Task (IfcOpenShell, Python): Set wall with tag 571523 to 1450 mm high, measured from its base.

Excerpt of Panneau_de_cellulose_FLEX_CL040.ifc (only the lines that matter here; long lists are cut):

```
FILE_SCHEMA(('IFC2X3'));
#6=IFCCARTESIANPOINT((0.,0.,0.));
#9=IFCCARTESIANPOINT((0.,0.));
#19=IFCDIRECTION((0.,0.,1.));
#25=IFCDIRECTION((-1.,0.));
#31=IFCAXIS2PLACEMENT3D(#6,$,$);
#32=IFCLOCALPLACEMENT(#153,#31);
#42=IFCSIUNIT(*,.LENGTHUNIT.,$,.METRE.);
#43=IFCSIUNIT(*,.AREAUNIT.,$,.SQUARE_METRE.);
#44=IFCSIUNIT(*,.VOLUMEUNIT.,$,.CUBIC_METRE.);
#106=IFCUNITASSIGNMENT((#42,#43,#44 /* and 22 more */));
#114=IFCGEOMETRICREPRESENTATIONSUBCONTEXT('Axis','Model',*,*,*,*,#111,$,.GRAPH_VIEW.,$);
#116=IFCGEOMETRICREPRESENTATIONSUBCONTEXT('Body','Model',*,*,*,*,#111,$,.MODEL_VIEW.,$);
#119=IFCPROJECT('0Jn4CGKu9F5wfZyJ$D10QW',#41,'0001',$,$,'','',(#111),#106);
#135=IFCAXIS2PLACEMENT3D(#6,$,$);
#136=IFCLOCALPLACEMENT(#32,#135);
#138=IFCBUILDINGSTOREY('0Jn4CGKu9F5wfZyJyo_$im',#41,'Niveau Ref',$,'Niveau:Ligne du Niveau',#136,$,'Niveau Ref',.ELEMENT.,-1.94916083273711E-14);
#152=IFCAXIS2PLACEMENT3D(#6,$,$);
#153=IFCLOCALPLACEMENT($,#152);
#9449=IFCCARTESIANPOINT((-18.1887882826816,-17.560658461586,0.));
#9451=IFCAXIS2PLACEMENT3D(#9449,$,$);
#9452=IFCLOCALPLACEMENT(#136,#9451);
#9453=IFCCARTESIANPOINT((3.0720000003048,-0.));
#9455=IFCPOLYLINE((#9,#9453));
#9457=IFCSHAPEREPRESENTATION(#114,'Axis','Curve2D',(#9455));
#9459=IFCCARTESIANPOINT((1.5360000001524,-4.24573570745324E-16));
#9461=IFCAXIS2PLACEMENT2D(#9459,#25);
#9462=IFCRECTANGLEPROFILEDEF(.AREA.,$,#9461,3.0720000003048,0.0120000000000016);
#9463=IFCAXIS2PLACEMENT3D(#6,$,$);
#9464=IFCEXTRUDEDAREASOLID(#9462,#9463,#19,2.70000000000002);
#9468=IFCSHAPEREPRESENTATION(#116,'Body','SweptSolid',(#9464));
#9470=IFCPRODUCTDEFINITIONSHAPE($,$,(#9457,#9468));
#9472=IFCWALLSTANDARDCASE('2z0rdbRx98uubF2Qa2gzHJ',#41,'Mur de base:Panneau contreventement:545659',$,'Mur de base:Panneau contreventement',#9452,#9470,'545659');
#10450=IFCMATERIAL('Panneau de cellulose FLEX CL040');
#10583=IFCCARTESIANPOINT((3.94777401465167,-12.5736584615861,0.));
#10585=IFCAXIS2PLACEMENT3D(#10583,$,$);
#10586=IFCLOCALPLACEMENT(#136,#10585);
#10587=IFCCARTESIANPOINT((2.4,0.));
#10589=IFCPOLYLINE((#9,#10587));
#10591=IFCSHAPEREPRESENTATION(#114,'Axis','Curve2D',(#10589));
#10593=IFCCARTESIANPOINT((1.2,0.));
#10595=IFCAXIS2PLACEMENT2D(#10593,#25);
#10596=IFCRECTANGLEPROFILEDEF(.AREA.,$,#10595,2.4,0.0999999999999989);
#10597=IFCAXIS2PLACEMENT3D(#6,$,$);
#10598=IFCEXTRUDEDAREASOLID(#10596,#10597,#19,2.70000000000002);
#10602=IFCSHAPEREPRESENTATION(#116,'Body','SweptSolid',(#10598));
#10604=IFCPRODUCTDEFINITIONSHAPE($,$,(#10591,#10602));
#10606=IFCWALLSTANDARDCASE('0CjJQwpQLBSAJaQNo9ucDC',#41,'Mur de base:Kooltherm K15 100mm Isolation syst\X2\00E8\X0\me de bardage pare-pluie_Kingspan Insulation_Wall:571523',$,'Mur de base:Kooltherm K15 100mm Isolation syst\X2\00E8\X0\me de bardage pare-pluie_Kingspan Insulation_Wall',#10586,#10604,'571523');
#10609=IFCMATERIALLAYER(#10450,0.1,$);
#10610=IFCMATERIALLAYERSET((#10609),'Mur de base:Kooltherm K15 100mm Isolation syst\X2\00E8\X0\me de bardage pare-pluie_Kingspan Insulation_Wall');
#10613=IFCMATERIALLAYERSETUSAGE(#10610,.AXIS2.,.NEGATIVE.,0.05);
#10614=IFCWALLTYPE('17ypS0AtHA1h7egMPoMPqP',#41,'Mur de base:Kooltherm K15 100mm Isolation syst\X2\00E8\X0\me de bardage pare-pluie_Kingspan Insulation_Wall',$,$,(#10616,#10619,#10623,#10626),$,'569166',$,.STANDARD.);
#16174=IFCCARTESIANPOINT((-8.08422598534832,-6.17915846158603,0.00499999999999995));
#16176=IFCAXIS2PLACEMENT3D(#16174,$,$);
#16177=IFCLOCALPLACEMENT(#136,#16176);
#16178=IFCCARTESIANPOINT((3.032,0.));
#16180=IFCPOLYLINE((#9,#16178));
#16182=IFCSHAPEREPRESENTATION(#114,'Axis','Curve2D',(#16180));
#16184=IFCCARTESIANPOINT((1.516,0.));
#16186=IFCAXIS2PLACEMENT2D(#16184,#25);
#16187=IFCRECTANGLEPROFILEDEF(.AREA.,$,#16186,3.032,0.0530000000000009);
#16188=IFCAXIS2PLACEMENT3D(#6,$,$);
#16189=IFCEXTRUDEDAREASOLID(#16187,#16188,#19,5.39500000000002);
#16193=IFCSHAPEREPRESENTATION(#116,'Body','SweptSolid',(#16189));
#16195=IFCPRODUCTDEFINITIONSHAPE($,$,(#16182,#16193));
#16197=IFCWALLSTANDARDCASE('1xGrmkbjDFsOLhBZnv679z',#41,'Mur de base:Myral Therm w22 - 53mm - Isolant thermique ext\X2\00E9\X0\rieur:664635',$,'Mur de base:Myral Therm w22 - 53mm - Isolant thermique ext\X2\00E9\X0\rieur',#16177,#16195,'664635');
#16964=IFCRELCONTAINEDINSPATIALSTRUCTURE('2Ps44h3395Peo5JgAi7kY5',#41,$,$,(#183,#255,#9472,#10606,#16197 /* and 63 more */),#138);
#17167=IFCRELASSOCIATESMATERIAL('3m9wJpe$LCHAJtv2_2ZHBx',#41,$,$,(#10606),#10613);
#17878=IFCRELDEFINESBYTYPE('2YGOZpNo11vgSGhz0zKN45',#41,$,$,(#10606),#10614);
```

```python
import ifcopenshell
import ifcopenshell.geom
import ifcopenshell.util.representation
import ifcopenshell.util.shape

model = ifcopenshell.open("Panneau_de_cellulose_FLEX_CL040.ifc")
settings = ifcopenshell.geom.settings()


def volume(element):
    """Net volume in cubic metres, openings subtracted."""
    shape = ifcopenshell.geom.create_shape(settings, element)
    return ifcopenshell.util.shape.get_volume(shape.geometry)


wall = model.by_id(10606)
before = volume(wall)

body = ifcopenshell.util.representation.get_representation(wall, "Model", "Body")
solid = body.Items[0]
old_height = solid.Depth
solid.Depth = 1.45
after = volume(wall)

print(f"height {old_height:g} -> {solid.Depth:g}, volume {before:.3f} -> {after:.3f} m3")

model.write("Panneau_de_cellulose_FLEX_CL040_rev.ifc")
```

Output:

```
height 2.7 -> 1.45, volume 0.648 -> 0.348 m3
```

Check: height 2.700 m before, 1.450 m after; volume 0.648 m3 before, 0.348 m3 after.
